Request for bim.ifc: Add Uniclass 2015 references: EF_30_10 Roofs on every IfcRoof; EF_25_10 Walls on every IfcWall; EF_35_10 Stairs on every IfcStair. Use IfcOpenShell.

First a look at what the model holds.

```python
import ifcopenshell

model = ifcopenshell.open("bim.ifc")
print(model.schema)
print("classifications:", [c.Name for c in model.by_type("IfcClassification")])
for ifc_class in ("IfcDoor", "IfcRoof", "IfcStair", "IfcWall", "IfcWindow"):
    print(ifc_class, len(model.by_type(ifc_class)))
```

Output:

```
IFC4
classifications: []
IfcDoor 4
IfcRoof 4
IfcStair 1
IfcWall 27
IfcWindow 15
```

```python
import ifcopenshell
import ifcopenshell.api.classification

model = ifcopenshell.open("bim.ifc")

system = ifcopenshell.api.classification.add_classification(model, classification="Uniclass 2015")

codes = {
    "IfcRoof": ("EF_30_10", "Roofs"),
    "IfcWall": ("EF_25_10", "Walls"),
    "IfcStair": ("EF_35_10", "Stairs"),
}
for ifc_class, (code, name) in codes.items():
    products = model.by_type(ifc_class)
    ifcopenshell.api.classification.add_reference(
        model, products=products, classification=system, identification=code, name=name
    )
    print(code, len(products))

model.write("bim-out.ifc")
```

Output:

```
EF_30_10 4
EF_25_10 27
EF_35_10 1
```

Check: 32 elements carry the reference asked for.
